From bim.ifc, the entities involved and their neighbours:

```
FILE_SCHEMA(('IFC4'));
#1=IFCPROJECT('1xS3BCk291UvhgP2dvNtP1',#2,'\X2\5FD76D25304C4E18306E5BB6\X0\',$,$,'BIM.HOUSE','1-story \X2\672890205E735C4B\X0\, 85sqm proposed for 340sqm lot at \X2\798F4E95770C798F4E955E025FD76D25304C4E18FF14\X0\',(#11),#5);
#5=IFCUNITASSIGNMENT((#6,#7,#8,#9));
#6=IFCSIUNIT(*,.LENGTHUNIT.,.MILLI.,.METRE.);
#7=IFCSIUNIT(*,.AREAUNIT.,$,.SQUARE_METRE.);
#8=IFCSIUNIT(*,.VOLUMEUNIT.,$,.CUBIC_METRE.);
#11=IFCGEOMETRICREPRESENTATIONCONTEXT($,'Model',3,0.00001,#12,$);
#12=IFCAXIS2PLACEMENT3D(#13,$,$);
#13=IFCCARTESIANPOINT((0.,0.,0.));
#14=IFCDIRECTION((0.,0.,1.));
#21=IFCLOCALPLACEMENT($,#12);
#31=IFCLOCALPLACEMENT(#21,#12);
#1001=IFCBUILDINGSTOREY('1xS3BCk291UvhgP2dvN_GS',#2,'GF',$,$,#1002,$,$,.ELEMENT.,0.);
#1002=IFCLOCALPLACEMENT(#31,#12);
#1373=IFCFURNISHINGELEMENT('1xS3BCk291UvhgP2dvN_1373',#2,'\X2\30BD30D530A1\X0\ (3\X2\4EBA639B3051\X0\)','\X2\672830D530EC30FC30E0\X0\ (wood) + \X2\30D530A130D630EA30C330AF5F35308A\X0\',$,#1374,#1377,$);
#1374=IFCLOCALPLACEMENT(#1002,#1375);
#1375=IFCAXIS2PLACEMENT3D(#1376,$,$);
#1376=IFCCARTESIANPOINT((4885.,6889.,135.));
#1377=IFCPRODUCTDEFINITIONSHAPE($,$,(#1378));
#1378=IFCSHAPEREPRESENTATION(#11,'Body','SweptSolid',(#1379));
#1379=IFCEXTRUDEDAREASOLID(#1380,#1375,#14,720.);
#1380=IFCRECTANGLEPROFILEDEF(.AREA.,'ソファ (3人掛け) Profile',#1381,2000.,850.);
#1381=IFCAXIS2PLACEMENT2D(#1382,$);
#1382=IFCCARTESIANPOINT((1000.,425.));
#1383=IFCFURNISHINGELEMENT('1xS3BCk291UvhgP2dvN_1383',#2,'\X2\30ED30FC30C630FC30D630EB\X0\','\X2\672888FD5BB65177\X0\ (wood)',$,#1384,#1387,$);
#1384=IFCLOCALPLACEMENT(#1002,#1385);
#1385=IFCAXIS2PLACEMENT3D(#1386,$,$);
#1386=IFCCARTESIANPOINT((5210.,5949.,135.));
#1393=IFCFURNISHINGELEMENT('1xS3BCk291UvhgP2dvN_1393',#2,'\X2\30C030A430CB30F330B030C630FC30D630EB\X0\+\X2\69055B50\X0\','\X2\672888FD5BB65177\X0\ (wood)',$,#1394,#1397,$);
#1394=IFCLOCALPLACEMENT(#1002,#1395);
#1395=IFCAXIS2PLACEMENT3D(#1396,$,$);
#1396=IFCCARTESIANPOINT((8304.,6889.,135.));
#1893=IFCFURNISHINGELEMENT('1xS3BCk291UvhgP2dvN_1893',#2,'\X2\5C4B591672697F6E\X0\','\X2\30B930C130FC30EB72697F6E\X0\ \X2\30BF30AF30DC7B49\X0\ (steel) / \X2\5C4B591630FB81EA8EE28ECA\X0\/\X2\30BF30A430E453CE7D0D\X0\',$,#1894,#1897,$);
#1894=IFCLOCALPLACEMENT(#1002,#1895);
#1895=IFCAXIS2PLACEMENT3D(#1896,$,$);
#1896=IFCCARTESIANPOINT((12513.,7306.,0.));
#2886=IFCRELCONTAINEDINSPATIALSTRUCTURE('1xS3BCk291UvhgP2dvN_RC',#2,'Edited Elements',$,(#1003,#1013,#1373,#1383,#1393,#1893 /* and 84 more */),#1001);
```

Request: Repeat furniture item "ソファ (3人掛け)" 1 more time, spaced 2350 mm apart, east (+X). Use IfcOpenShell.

```python
import numpy as np
import ifcopenshell
import ifcopenshell.api.geometry
import ifcopenshell.api.root
import ifcopenshell.util.element
import ifcopenshell.util.placement

model = ifcopenshell.open("bim.ifc")


def reuse_history(source, copy):
    """copy_class also copies each property set's owner history, people and application; keep the originals."""
    for rel in copy.IsDefinedBy:
        if rel.is_a("IfcRelDefinesByProperties") and (history := rel.RelatingPropertyDefinition.OwnerHistory):
            rel.RelatingPropertyDefinition.OwnerHistory = source.OwnerHistory
            ifcopenshell.util.element.remove_deep2(model, history)


source = model.by_id(1373)
base = ifcopenshell.util.placement.get_local_placement(source.ObjectPlacement)
step = np.array([1.0, 0.0, 0.0]) * 2350.0

for i in range(1, 2):
    copy = ifcopenshell.api.root.copy_class(model, product=source)
    copy.Representation = ifcopenshell.util.element.copy_deep(
        model, source.Representation, exclude=["IfcGeometricRepresentationContext", "IfcRepresentationMap"]
    )
    reuse_history(source, copy)
    matrix = base.copy()
    matrix[:3, 3] += i * step
    print("added at", matrix[:3, 3].round(3) + 0.0)
    ifcopenshell.api.geometry.edit_object_placement(model, product=copy, matrix=matrix, is_si=False)

model.write("bim_v2.ifc")
```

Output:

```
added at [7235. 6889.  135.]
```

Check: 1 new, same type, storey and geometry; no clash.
